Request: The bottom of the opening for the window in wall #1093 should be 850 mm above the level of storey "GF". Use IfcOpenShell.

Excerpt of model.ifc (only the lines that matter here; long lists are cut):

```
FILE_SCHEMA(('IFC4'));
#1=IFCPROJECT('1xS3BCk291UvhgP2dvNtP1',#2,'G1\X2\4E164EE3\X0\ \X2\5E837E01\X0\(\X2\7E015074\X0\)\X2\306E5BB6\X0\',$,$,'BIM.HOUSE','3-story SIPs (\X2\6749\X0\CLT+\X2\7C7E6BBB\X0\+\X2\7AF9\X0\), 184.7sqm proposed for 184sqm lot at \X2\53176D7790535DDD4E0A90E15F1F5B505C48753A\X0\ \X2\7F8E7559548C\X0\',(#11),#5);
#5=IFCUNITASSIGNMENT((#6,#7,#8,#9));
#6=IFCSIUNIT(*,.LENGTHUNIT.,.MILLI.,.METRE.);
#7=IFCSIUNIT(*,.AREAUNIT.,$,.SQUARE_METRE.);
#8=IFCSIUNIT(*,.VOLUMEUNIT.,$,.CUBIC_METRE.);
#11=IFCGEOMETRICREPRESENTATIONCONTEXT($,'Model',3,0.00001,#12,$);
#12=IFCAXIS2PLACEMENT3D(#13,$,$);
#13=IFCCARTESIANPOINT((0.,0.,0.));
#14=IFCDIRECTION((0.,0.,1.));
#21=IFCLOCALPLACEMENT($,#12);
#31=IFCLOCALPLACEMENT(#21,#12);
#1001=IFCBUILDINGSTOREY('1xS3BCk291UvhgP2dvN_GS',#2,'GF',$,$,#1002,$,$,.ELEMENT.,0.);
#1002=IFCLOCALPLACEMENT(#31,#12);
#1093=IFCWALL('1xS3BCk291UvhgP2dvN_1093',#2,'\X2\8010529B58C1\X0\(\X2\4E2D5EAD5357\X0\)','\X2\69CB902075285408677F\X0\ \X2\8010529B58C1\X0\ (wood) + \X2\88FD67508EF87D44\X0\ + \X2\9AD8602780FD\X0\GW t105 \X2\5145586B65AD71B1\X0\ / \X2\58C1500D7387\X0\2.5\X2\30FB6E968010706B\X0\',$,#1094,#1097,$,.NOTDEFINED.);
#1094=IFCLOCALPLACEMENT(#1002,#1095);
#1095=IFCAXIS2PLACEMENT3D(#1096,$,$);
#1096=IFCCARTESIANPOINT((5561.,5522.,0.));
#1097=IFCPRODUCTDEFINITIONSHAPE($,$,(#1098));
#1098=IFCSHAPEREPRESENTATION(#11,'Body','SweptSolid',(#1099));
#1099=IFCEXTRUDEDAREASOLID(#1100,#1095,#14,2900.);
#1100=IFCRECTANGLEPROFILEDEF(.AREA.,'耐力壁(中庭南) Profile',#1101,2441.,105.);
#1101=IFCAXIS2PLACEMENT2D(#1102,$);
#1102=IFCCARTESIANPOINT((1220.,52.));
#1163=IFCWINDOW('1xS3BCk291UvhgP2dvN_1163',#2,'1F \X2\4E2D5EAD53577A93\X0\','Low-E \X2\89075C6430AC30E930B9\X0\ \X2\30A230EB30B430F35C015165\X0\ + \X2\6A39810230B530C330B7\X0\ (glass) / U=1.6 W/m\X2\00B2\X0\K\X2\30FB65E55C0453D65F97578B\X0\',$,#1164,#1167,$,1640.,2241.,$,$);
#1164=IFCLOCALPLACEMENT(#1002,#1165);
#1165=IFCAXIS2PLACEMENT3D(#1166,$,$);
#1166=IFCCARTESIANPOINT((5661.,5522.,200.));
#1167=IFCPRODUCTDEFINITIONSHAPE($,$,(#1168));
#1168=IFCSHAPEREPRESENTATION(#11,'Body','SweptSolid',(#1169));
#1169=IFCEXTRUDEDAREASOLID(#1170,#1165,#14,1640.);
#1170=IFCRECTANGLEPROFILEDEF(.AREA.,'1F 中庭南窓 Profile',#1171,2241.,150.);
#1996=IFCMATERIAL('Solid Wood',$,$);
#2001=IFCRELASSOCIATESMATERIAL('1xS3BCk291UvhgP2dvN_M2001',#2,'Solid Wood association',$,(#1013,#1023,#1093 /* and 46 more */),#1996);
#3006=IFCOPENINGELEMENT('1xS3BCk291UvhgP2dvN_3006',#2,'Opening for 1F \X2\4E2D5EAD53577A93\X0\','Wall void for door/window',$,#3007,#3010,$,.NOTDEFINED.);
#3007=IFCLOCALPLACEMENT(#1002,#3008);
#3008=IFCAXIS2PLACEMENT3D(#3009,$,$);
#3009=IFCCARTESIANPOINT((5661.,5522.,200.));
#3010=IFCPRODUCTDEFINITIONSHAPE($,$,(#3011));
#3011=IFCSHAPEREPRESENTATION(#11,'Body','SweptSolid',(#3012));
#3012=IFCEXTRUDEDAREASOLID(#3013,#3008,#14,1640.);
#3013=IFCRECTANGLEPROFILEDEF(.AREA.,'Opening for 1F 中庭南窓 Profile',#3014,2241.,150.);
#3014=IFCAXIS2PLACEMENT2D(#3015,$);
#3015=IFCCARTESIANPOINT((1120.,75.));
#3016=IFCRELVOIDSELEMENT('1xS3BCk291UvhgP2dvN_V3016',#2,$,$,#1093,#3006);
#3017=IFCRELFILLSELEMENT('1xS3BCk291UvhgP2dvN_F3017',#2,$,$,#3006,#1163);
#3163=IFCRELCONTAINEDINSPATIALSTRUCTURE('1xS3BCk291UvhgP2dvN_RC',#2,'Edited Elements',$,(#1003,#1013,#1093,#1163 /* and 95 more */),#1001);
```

```python
import numpy as np
import ifcopenshell
import ifcopenshell.api.geometry
import ifcopenshell.geom
import ifcopenshell.util.element
import ifcopenshell.util.placement
import ifcopenshell.util.shape
import ifcopenshell.util.unit

model = ifcopenshell.open("model.ifc")
unit_scale = ifcopenshell.util.unit.calculate_unit_scale(model)

window = model.by_guid("1xS3BCk291UvhgP2dvN_1163")
opening = window.FillsVoids[0].RelatingOpeningElement
storey = ifcopenshell.util.element.get_container(window, ifc_class="IfcBuildingStorey")
level = ifcopenshell.util.placement.get_local_placement(storey.ObjectPlacement)[2, 3]

# The opening's origin need not be at the sill, so measure its lowest point.
shape = ifcopenshell.geom.create_shape(ifcopenshell.geom.settings(), opening)
bottom = ifcopenshell.util.shape.get_shape_bottom_elevation(shape, shape.geometry) / unit_scale
dz = level + 850.0 - bottom

shift = np.array([0.0, 0.0, dz])
# The window is not placed relative to its opening, so move both.
for product in (opening, window):
    matrix = ifcopenshell.util.placement.get_local_placement(product.ObjectPlacement)
    matrix[:3, 3] += shift
    ifcopenshell.api.geometry.edit_object_placement(model, product=product, matrix=matrix, is_si=False)

print(f"moved by {dz * unit_scale:+.3f} m")

model.write("model_rev.ifc")
```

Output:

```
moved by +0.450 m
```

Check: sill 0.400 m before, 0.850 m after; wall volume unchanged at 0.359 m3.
